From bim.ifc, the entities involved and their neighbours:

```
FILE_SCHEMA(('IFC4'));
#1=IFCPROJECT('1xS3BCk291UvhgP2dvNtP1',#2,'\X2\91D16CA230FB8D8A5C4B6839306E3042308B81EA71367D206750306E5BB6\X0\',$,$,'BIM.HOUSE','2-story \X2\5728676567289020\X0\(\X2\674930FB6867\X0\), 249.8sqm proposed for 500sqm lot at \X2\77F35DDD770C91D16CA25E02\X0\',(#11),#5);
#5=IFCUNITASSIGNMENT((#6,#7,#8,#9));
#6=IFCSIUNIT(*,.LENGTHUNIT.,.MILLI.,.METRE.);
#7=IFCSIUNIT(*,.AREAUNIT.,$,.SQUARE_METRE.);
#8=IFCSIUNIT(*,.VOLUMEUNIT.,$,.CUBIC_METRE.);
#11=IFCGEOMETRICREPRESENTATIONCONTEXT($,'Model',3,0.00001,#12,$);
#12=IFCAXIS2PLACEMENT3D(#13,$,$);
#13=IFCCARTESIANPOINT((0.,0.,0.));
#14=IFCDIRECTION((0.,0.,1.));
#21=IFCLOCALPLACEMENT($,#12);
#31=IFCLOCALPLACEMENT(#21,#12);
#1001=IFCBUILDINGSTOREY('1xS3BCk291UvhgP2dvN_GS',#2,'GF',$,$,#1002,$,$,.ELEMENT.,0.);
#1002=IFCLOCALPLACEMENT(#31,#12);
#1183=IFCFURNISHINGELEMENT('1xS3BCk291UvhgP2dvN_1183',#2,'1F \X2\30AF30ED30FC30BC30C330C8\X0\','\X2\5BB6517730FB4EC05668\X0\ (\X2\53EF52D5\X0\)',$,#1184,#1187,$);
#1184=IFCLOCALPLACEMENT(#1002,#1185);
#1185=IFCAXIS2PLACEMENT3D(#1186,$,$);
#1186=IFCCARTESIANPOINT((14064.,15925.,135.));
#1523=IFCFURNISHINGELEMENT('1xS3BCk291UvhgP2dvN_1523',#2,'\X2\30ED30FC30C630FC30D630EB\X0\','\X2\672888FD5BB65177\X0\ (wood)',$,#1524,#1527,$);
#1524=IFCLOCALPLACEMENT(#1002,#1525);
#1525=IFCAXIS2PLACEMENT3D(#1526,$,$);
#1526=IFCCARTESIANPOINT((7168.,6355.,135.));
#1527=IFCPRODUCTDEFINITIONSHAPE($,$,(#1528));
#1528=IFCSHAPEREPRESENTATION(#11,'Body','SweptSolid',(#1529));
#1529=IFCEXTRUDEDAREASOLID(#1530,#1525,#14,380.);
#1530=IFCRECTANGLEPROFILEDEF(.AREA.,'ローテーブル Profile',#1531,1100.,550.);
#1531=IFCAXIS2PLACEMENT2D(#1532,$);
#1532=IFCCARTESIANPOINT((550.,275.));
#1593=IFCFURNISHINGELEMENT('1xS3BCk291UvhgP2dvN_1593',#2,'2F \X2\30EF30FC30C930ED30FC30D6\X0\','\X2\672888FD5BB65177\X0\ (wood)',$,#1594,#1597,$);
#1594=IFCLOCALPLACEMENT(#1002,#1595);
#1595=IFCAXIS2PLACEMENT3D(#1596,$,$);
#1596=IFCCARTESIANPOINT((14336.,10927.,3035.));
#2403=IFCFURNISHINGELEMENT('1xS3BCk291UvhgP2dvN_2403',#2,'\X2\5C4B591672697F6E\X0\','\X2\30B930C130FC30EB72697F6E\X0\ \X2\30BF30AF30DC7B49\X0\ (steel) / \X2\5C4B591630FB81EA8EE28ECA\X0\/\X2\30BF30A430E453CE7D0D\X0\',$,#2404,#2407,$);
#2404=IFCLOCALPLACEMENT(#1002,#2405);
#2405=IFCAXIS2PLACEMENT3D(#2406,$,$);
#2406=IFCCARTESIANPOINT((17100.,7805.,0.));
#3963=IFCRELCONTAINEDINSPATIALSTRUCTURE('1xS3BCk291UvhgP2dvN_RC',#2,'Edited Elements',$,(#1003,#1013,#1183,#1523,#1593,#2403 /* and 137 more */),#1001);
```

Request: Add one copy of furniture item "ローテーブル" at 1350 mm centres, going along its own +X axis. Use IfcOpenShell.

```python
import ifcopenshell
import ifcopenshell.api.geometry
import ifcopenshell.api.root
import ifcopenshell.util.element
import ifcopenshell.util.placement
import ifcopenshell.util.unit

model = ifcopenshell.open("bim.ifc")
unit_scale = ifcopenshell.util.unit.calculate_unit_scale(model)


def reuse_history(source, copy):
    """copy_class also copies each property set's owner history, people and application; keep the originals."""
    for rel in copy.IsDefinedBy:
        if rel.is_a("IfcRelDefinesByProperties") and (history := rel.RelatingPropertyDefinition.OwnerHistory):
            rel.RelatingPropertyDefinition.OwnerHistory = source.OwnerHistory
            ifcopenshell.util.element.remove_deep2(model, history)


source = model.by_guid("1xS3BCk291UvhgP2dvN_1523")
base = ifcopenshell.util.placement.get_local_placement(source.ObjectPlacement)
step = base[:3, 0] * 1.35 / unit_scale

for i in range(1, 2):
    copy = ifcopenshell.api.root.copy_class(model, product=source)
    copy.Representation = ifcopenshell.util.element.copy_deep(
        model, source.Representation, exclude=["IfcGeometricRepresentationContext", "IfcRepresentationMap"]
    )
    reuse_history(source, copy)
    matrix = base.copy()
    matrix[:3, 3] += i * step
    print("added at", matrix[:3, 3].round(3) + 0.0)
    ifcopenshell.api.geometry.edit_object_placement(model, product=copy, matrix=matrix, is_si=False)

model.write("bim_v2.ifc")
```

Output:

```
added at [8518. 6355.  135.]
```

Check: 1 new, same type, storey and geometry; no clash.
